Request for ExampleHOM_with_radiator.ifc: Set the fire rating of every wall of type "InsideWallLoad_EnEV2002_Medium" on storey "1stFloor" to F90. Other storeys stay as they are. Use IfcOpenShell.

First a look at what the model holds.

```python
import ifcopenshell
import ifcopenshell.util.element

model = ifcopenshell.open("ExampleHOM_with_radiator.ifc")
print(model.schema)
storey = next(s for s in model.by_type("IfcBuildingStorey") if s.Name == "1stFloor")
walls = [e for e in ifcopenshell.util.element.get_decomposition(storey) if e.is_a("IfcWall")]
seen = {}
for e in walls:
    element_type = ifcopenshell.util.element.get_type(e)
    key = (element_type.Name if element_type != e and element_type else None, ifcopenshell.util.element.get_pset(e, "Pset_WallCommon", "FireRating"))
    seen[key] = seen.get(key, 0) + 1
for (name, value), count in sorted(seen.items(), key=str):
    print(count, "x", name, "|", value)
```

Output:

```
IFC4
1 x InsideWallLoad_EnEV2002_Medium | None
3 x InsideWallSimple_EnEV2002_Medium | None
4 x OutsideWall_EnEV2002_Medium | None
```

```python
import ifcopenshell
import ifcopenshell.api.pset
import ifcopenshell.util.element

model = ifcopenshell.open("ExampleHOM_with_radiator.ifc")

storey = next(s for s in model.by_type("IfcBuildingStorey") if s.Name == "1stFloor")
walls = [e for e in ifcopenshell.util.element.get_decomposition(storey) if e.is_a("IfcWall")]

count = 0
for e in walls:
    element_type = ifcopenshell.util.element.get_type(e)
    if element_type in (None, e) or element_type.Name != "InsideWallLoad_EnEV2002_Medium":
        continue
    # add_pset returns the element's existing set when there is one.
    pset = ifcopenshell.api.pset.add_pset(model, product=e, name="Pset_WallCommon")
    ifcopenshell.api.pset.edit_pset(model, pset=pset, properties={"FireRating": "F90"})
    count += 1

print(count, "walls updated")

model.write("ExampleHOM_with_radiator_v2.ifc")
```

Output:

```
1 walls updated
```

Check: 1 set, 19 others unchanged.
